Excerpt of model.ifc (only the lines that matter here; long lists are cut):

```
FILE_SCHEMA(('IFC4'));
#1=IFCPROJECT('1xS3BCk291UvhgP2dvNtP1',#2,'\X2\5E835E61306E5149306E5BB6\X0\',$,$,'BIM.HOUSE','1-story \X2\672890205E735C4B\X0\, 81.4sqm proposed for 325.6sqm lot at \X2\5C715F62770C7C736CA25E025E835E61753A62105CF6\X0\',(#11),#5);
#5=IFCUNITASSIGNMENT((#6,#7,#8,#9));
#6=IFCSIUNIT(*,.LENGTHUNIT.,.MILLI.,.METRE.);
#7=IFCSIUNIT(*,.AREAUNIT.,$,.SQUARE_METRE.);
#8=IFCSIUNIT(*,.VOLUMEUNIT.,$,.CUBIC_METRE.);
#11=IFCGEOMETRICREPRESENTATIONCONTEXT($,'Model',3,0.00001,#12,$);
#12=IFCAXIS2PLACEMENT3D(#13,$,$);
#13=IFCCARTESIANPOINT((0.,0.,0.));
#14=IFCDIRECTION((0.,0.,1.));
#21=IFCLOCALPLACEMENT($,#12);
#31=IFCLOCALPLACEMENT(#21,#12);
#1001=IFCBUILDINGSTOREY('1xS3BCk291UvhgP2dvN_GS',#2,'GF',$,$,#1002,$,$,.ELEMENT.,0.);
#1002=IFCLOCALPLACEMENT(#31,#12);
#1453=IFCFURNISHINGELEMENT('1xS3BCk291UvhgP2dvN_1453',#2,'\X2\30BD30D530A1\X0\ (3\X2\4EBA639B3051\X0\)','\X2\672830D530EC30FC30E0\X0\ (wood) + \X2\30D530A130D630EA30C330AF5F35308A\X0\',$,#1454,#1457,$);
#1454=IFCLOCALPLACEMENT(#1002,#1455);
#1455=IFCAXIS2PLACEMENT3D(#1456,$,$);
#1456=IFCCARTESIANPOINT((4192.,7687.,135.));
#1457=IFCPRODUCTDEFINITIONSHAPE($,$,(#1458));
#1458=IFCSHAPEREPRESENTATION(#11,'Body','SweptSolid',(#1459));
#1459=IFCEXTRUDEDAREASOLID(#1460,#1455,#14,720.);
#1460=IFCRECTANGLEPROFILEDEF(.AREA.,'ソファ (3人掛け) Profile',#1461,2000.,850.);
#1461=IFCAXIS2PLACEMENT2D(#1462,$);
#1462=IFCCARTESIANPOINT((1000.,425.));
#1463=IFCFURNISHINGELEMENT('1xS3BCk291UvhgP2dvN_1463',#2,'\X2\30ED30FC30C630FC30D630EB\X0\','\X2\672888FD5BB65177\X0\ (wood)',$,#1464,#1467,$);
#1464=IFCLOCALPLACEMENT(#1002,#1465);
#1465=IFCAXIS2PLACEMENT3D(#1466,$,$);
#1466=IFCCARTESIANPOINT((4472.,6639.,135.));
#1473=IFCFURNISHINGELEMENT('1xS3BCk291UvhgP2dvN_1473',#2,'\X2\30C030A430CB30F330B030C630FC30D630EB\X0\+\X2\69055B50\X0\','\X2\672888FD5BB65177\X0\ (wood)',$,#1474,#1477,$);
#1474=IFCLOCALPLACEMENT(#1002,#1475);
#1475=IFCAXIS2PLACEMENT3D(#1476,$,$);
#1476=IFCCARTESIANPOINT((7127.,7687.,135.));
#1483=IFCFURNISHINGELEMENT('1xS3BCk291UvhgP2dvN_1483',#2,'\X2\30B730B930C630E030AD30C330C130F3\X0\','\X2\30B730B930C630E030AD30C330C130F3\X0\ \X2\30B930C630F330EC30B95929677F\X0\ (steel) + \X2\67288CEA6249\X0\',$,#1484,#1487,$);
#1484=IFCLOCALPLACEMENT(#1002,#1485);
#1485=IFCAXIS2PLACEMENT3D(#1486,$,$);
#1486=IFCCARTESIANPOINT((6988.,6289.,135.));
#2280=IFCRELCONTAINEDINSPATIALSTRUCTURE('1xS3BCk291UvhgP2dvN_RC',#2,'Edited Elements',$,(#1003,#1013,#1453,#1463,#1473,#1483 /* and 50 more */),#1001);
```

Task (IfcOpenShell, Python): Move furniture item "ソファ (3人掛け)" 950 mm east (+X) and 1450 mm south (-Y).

```python
import ifcopenshell
import ifcopenshell.api.geometry
import ifcopenshell.util.placement
import ifcopenshell.util.unit

model = ifcopenshell.open("model.ifc")
unit_scale = ifcopenshell.util.unit.calculate_unit_scale(model)

item = model.by_guid("1xS3BCk291UvhgP2dvN_1453")
matrix = ifcopenshell.util.placement.get_local_placement(item.ObjectPlacement)
matrix[0, 3] += 0.95 / unit_scale
matrix[1, 3] -= 1.45 / unit_scale
ifcopenshell.api.geometry.edit_object_placement(model, product=item, matrix=matrix, is_si=False)

print(ifcopenshell.util.placement.get_local_placement(item.ObjectPlacement).round(3) + 0.0)

model.write("model_edited.ifc")
```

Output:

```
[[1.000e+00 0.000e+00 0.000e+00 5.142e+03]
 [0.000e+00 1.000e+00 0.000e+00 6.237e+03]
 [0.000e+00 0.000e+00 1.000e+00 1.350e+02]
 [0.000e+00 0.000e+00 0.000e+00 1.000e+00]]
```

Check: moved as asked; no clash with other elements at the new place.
